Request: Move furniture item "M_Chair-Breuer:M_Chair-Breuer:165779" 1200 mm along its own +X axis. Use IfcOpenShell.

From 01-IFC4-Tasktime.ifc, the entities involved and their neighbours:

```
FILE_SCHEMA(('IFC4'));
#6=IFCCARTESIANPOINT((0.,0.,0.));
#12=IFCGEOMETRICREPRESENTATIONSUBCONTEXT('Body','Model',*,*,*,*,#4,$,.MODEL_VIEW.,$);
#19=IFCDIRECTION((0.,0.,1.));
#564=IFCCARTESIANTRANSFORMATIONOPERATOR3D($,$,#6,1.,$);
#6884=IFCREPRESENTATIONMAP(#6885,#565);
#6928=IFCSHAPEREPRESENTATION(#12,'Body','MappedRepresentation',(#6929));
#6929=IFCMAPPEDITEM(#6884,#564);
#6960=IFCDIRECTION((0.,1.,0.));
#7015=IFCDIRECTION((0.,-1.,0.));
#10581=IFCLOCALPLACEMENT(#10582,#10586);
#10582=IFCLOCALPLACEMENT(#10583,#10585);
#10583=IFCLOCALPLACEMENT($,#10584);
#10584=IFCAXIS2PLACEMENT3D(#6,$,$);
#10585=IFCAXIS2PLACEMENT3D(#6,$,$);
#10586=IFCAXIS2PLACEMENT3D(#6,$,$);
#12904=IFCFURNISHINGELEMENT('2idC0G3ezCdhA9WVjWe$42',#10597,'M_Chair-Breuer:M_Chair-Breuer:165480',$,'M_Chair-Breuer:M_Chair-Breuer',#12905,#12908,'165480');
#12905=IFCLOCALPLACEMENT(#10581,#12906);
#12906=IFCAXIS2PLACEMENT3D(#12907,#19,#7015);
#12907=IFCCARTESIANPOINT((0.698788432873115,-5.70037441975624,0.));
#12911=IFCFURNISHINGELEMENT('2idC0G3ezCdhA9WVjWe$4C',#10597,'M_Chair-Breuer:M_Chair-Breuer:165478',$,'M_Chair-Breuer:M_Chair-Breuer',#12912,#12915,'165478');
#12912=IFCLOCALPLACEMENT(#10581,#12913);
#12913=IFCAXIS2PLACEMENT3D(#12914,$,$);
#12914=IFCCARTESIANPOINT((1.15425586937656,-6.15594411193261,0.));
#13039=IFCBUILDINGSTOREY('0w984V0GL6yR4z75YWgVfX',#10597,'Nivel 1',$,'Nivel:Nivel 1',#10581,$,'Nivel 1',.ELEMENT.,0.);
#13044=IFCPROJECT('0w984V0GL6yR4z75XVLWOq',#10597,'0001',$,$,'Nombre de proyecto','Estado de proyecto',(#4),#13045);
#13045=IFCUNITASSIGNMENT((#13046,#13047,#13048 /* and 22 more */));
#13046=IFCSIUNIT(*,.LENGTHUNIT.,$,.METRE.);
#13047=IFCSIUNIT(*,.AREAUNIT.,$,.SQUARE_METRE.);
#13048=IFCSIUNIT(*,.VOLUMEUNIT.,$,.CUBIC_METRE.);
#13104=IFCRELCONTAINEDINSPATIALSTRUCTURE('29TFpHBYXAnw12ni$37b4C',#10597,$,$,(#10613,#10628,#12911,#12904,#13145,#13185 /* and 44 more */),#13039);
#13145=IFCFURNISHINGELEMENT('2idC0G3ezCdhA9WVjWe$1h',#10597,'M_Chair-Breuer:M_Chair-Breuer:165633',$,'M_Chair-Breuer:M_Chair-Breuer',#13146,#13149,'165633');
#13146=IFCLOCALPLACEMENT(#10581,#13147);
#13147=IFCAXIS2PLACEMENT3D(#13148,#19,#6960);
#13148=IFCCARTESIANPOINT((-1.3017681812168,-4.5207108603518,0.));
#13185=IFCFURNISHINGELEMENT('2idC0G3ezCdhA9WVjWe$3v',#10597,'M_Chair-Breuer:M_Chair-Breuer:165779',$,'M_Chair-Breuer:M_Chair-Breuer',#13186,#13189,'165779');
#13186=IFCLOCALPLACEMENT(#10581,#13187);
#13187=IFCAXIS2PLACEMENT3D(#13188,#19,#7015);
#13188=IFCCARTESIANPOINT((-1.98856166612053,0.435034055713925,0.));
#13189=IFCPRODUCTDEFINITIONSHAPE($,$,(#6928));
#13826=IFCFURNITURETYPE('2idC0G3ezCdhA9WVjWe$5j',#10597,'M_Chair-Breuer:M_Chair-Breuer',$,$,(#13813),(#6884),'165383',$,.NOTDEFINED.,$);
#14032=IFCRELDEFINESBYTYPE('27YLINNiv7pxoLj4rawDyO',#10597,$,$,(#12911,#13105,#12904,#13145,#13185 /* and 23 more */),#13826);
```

```python
import ifcopenshell
import ifcopenshell.api.geometry
import ifcopenshell.util.placement
import ifcopenshell.util.unit

model = ifcopenshell.open("01-IFC4-Tasktime.ifc")
unit_scale = ifcopenshell.util.unit.calculate_unit_scale(model)

item = model.by_id(13185)
matrix = ifcopenshell.util.placement.get_local_placement(item.ObjectPlacement)
matrix[:3, 3] += matrix[:3, 0] * 1.2 / unit_scale
ifcopenshell.api.geometry.edit_object_placement(model, product=item, matrix=matrix, is_si=False)

print(ifcopenshell.util.placement.get_local_placement(item.ObjectPlacement).round(3) + 0.0)

model.write("01-IFC4-Tasktime_updated.ifc")
```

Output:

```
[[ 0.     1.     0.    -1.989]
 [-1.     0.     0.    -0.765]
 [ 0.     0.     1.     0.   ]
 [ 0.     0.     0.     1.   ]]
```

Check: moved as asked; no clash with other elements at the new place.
